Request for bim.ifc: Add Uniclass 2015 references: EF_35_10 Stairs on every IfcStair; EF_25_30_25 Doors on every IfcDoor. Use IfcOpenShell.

First a look at what the model holds.

```python
import ifcopenshell

model = ifcopenshell.open("bim.ifc")
print(model.schema)
print("classifications:", [c.Name for c in model.by_type("IfcClassification")])
for ifc_class in ("IfcDoor", "IfcRoof", "IfcStair", "IfcWall", "IfcWindow"):
    print(ifc_class, len(model.by_type(ifc_class)))
```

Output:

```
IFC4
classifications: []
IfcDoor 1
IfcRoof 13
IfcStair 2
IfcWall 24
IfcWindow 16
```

```python
import ifcopenshell
import ifcopenshell.api.classification

model = ifcopenshell.open("bim.ifc")

system = ifcopenshell.api.classification.add_classification(model, classification="Uniclass 2015")

codes = {
    "IfcStair": ("EF_35_10", "Stairs"),
    "IfcDoor": ("EF_25_30_25", "Doors"),
}
for ifc_class, (code, name) in codes.items():
    products = model.by_type(ifc_class)
    ifcopenshell.api.classification.add_reference(
        model, products=products, classification=system, identification=code, name=name
    )
    print(code, len(products))

model.write("bim_edited.ifc")
```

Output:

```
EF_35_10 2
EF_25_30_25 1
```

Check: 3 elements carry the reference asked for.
